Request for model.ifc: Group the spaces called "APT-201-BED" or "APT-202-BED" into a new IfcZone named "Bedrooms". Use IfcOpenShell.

First a look at what the model holds.

```python
import ifcopenshell

model = ifcopenshell.open("model.ifc")
print(model.schema)
seen = {}
for space in model.by_type("IfcSpace"):
    seen[space.Name] = seen.get(space.Name, 0) + 1
for name, count in sorted(seen.items(), key=str):
    print(count, "x", name)
print("zones:", [z.Name for z in model.by_type("IfcZone")][:20])
```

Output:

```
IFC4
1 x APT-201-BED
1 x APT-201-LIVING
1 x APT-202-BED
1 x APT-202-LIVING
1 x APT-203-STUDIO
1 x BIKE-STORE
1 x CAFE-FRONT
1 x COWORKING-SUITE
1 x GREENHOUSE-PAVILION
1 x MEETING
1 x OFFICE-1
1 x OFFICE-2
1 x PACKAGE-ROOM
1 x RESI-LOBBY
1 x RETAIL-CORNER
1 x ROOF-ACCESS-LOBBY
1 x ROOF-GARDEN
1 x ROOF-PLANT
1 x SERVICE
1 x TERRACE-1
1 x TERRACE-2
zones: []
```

```python
import ifcopenshell
import ifcopenshell.api.group
import ifcopenshell.api.root

model = ifcopenshell.open("model.ifc")

names = {"APT-201-BED", "APT-202-BED"}
spaces = [s for s in model.by_type("IfcSpace") if s.Name in names]

zone = ifcopenshell.api.root.create_entity(model, ifc_class="IfcZone", name="Bedrooms")
ifcopenshell.api.group.assign_group(model, products=spaces, group=zone)
print(len(spaces), "spaces in", zone.Name)

model.write("model_updated.ifc")
```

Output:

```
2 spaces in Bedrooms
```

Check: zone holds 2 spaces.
